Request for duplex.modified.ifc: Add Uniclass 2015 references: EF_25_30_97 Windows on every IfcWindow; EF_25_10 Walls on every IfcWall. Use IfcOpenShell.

First a look at what the model holds.

```python
import ifcopenshell

model = ifcopenshell.open("duplex.modified.ifc")
print(model.schema)
print("classifications:", [c.Name for c in model.by_type("IfcClassification")])
for ifc_class in ("IfcDoor", "IfcRoof", "IfcStair", "IfcWall", "IfcWindow"):
    print(ifc_class, len(model.by_type(ifc_class)))
```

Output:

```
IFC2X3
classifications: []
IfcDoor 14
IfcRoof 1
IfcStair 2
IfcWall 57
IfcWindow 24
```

```python
import ifcopenshell
import ifcopenshell.api.classification

model = ifcopenshell.open("duplex.modified.ifc")

# IFC2X3 requires Source and Edition and has no link from the project to the system.
system = model.create_entity("IfcClassification", Source="NBS", Edition="2015", Name="Uniclass 2015")

codes = {
    "IfcWindow": ("EF_25_30_97", "Windows"),
    "IfcWall": ("EF_25_10", "Walls"),
}
for ifc_class, (code, name) in codes.items():
    products = model.by_type(ifc_class)
    ifcopenshell.api.classification.add_reference(
        model, products=products, classification=system, identification=code, name=name
    )
    print(code, len(products))

model.write("duplex.modified-out.ifc")
```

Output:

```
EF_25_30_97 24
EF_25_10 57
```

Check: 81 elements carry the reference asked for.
